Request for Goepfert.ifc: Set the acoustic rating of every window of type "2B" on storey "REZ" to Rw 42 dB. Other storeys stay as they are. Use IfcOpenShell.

First a look at what the model holds.

```python
import ifcopenshell
import ifcopenshell.util.element

model = ifcopenshell.open("Goepfert.ifc")
print(model.schema)
storey = next(s for s in model.by_type("IfcBuildingStorey") if s.Name == "REZ")
windows = [e for e in ifcopenshell.util.element.get_decomposition(storey) if e.is_a("IfcWindow")]
seen = {}
for e in windows:
    element_type = ifcopenshell.util.element.get_type(e)
    key = (element_type.Name if element_type != e and element_type else None, ifcopenshell.util.element.get_pset(e, "Pset_WindowCommon", "AcousticRating"))
    seen[key] = seen.get(key, 0) + 1
for (name, value), count in sorted(seen.items(), key=str):
    print(count, "x", name, "|", value)
```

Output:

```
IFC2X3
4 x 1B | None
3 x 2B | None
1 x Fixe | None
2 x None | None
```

```python
import ifcopenshell
import ifcopenshell.api.pset
import ifcopenshell.util.element

model = ifcopenshell.open("Goepfert.ifc")

storey = next(s for s in model.by_type("IfcBuildingStorey") if s.Name == "REZ")
windows = [e for e in ifcopenshell.util.element.get_decomposition(storey) if e.is_a("IfcWindow")]

count = 0
for e in windows:
    element_type = ifcopenshell.util.element.get_type(e)
    if element_type in (None, e) or element_type.Name != "2B":
        continue
    # add_pset returns the element's existing set when there is one.
    pset = ifcopenshell.api.pset.add_pset(model, product=e, name="Pset_WindowCommon")
    ifcopenshell.api.pset.edit_pset(model, pset=pset, properties={"AcousticRating": "Rw 42 dB"})
    count += 1

print(count, "windows updated")

model.write("Goepfert_v2.ifc")
```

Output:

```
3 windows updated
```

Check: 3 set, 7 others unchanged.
